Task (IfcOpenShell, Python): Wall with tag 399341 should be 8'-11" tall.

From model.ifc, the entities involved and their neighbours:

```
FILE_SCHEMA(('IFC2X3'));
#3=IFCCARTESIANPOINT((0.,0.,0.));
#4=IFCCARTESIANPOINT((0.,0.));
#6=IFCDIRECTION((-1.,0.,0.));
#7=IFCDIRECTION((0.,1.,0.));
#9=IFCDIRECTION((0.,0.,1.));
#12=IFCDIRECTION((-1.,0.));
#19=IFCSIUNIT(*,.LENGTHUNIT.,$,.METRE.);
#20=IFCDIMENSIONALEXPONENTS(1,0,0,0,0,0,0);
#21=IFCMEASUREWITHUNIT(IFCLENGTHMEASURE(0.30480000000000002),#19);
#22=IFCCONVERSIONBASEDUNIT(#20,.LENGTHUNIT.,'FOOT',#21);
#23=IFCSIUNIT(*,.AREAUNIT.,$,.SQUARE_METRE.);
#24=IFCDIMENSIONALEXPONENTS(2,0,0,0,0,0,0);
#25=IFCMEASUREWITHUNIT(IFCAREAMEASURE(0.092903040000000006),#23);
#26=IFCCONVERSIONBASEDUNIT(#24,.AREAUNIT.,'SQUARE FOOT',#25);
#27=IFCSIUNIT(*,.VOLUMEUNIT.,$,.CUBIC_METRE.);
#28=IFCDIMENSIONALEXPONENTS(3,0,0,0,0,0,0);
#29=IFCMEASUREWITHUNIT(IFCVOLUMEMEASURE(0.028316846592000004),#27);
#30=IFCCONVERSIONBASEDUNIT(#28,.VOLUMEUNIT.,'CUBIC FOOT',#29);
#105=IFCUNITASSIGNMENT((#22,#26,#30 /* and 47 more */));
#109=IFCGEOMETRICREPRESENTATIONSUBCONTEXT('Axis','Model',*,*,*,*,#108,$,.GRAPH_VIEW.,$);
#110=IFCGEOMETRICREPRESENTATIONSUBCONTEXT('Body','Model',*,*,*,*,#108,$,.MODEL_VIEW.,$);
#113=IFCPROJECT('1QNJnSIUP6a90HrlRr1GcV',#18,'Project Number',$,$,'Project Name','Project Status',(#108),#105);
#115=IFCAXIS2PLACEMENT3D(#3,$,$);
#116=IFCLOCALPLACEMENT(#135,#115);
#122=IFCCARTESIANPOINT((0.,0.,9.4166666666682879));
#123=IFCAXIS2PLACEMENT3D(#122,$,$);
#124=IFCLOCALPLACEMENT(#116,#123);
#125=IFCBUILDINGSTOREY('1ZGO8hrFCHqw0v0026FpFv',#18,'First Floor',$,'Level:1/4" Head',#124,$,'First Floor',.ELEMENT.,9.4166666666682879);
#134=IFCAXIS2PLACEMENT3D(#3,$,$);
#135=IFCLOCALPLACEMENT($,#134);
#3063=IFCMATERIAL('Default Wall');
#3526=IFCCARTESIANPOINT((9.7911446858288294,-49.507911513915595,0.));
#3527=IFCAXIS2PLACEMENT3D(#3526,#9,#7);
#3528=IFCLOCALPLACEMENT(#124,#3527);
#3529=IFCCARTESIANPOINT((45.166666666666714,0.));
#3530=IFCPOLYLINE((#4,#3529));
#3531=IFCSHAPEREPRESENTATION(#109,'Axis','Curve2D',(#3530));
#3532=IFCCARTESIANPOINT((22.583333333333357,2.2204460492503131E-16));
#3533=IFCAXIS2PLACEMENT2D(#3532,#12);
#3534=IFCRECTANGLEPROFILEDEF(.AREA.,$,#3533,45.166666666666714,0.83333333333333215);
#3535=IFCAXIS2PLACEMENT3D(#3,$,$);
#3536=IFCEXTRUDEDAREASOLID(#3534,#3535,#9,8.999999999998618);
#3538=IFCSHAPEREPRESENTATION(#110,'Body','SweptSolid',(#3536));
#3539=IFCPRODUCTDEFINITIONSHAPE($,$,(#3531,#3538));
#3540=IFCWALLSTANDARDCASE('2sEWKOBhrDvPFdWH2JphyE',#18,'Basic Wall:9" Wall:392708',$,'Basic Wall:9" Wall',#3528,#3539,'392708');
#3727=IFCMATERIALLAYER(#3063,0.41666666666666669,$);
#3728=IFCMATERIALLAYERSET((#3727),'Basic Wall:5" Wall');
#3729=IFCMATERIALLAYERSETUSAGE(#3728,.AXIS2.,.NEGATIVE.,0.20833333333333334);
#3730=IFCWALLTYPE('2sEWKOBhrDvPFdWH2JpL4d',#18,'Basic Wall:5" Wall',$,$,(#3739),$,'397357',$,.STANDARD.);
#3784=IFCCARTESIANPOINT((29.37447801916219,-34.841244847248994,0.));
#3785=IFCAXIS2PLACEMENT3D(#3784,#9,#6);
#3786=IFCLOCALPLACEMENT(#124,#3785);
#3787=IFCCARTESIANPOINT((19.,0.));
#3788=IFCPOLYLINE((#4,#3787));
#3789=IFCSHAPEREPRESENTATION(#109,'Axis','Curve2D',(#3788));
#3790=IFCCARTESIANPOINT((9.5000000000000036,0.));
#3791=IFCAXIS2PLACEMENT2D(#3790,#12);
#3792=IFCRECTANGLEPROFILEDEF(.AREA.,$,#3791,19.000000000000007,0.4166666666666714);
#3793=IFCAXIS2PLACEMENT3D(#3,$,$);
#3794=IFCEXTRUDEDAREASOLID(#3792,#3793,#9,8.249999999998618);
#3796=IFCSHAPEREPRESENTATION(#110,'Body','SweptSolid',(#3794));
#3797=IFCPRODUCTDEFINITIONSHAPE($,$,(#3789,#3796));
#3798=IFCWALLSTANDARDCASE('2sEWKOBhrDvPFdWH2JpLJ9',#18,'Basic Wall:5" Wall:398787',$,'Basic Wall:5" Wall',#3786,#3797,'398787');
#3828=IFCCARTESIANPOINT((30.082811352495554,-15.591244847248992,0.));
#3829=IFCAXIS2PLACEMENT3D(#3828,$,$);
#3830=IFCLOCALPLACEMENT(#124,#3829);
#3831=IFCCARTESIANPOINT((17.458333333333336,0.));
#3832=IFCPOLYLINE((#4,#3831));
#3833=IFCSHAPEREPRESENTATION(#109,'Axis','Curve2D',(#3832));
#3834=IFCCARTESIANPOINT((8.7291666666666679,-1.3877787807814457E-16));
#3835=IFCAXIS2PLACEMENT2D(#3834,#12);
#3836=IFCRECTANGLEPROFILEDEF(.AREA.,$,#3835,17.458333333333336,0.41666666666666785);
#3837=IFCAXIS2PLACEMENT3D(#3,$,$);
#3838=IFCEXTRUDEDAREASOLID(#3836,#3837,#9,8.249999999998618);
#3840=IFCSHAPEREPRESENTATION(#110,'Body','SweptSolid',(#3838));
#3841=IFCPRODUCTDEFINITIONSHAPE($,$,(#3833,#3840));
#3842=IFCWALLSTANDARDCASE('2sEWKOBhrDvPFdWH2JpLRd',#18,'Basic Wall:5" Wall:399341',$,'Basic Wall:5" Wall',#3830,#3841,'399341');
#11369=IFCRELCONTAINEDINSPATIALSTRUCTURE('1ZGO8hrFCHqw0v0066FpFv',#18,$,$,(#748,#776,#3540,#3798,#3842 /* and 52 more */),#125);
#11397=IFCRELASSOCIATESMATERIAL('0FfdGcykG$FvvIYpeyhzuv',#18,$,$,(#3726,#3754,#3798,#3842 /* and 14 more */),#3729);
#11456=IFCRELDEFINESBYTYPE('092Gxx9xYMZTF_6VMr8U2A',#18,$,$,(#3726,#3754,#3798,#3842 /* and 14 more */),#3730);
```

```python
import ifcopenshell
import ifcopenshell.geom
import ifcopenshell.util.representation
import ifcopenshell.util.shape
import ifcopenshell.util.unit

model = ifcopenshell.open("model.ifc")
unit_scale = ifcopenshell.util.unit.calculate_unit_scale(model)
settings = ifcopenshell.geom.settings()


def volume(element):
    """Net volume in cubic metres, openings subtracted."""
    shape = ifcopenshell.geom.create_shape(settings, element)
    return ifcopenshell.util.shape.get_volume(shape.geometry)


wall = model.by_guid("2sEWKOBhrDvPFdWH2JpLRd")
before = volume(wall)

body = ifcopenshell.util.representation.get_representation(wall, "Model", "Body")
solid = body.Items[0]
old_height = solid.Depth
solid.Depth = 107 * 0.0254 / unit_scale
after = volume(wall)

print(f"height {old_height:g} -> {solid.Depth:g}, volume {before:.3f} -> {after:.3f} m3")

model.write("model_rev.ifc")
```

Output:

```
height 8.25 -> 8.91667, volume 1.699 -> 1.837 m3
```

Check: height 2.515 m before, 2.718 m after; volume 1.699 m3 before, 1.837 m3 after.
